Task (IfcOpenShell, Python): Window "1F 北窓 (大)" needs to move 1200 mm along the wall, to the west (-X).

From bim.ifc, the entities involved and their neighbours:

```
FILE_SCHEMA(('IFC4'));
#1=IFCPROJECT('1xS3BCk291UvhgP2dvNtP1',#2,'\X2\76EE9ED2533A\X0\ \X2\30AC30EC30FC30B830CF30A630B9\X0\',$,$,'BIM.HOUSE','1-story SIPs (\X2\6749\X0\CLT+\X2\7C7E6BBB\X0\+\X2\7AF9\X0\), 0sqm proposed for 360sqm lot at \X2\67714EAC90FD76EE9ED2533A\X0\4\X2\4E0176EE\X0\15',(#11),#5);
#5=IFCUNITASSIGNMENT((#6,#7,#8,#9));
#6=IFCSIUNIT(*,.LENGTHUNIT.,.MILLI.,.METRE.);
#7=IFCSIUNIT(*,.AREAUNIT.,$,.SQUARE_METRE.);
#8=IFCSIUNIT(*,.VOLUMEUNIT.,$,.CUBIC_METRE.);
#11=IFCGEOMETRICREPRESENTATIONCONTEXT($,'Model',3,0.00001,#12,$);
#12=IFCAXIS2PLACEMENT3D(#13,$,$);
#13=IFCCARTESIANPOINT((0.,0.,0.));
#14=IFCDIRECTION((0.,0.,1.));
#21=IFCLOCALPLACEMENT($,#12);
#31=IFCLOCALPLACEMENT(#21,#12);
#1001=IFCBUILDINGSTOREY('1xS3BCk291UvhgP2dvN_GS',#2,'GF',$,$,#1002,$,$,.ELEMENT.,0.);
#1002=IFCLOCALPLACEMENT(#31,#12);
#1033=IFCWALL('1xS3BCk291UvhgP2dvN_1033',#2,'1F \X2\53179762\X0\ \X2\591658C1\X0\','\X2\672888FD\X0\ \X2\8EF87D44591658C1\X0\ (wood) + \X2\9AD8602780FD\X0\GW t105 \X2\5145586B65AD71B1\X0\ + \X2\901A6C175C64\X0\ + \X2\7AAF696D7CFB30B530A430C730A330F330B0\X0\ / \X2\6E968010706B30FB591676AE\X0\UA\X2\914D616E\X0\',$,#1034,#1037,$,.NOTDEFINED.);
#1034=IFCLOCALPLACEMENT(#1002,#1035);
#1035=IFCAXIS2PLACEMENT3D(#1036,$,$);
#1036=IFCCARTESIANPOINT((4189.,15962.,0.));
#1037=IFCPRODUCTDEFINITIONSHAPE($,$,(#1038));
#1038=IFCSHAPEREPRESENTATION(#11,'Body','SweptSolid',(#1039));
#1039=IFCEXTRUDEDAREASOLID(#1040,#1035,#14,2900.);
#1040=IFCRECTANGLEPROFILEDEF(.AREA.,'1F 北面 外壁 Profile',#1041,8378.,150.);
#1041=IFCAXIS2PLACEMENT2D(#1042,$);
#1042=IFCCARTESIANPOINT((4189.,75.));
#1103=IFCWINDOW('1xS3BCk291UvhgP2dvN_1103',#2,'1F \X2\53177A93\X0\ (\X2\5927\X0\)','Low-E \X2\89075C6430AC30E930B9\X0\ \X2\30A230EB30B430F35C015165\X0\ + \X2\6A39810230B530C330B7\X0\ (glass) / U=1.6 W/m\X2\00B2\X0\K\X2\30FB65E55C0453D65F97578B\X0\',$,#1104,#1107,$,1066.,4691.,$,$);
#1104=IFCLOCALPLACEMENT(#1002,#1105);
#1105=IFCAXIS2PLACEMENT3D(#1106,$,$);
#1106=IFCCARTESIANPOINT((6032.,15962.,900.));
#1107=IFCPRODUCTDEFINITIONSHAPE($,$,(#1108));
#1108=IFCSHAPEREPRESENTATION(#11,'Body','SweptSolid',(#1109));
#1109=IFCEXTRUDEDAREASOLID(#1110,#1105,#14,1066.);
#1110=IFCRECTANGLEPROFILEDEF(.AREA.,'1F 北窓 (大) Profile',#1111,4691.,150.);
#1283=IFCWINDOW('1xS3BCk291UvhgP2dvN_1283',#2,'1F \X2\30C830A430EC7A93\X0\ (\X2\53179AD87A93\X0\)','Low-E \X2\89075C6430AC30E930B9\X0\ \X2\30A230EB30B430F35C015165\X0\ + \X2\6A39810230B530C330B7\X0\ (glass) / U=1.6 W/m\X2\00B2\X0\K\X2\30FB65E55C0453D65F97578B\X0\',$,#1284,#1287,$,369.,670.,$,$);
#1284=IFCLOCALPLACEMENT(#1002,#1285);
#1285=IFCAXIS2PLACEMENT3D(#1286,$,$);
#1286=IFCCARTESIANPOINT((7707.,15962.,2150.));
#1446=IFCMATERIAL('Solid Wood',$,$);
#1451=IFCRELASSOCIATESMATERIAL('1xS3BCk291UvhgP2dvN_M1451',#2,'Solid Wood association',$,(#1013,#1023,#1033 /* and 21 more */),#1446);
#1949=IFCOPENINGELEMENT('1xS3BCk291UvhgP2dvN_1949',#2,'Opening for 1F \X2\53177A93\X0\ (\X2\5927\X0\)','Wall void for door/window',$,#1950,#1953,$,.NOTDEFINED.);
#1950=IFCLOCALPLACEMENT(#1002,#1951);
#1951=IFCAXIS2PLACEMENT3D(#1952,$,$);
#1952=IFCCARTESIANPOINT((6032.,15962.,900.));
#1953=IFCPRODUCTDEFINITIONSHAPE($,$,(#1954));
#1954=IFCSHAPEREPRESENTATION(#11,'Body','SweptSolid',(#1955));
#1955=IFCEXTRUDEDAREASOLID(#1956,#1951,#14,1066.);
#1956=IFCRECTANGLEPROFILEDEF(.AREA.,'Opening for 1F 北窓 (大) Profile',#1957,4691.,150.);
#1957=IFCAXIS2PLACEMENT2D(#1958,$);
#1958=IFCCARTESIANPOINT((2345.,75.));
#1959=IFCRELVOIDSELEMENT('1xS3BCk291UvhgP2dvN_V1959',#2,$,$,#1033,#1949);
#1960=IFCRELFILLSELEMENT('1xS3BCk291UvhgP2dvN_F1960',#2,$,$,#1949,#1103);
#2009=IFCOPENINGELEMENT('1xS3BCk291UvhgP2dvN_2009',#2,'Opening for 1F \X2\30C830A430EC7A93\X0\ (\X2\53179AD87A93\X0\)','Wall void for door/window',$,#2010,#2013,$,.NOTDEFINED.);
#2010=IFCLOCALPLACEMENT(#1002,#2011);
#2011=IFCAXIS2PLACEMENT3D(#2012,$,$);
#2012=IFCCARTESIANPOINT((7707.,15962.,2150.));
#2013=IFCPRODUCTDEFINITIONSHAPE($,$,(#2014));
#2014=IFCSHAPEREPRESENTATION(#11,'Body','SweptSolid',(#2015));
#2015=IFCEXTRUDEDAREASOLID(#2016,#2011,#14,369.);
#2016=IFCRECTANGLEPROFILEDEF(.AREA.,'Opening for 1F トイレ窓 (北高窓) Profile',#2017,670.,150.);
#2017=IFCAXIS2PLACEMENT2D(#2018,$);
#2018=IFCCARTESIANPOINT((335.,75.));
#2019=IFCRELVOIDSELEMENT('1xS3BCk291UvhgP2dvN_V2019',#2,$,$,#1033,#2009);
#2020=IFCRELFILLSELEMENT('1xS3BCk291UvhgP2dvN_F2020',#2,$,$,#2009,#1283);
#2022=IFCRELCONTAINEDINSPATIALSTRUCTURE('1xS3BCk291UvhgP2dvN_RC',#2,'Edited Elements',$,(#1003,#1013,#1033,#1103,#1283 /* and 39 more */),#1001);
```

```python
import ifcopenshell
import ifcopenshell.api.geometry
import ifcopenshell.util.placement

model = ifcopenshell.open("bim.ifc")

window = model.by_guid("1xS3BCk291UvhgP2dvN_1103")
opening = window.FillsVoids[0].RelatingOpeningElement
wall = opening.VoidsElements[0].RelatingBuildingElement

wall_matrix = ifcopenshell.util.placement.get_local_placement(wall.ObjectPlacement)
shift = wall_matrix[:3, 0] * -1200.0
before = ifcopenshell.util.placement.get_local_placement(window.ObjectPlacement)[:3, 3].copy()

# The window is not placed relative to its opening, so move both.
for product in (opening, window):
    matrix = ifcopenshell.util.placement.get_local_placement(product.ObjectPlacement)
    matrix[:3, 3] += shift
    ifcopenshell.api.geometry.edit_object_placement(model, product=product, matrix=matrix, is_si=False)

after = ifcopenshell.util.placement.get_local_placement(window.ObjectPlacement)[:3, 3]
print("window moved by", (after - before).round(3) + 0.0)

model.write("bim_rev.ifc")
```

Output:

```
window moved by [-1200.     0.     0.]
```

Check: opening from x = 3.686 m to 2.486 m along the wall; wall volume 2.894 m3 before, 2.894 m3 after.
